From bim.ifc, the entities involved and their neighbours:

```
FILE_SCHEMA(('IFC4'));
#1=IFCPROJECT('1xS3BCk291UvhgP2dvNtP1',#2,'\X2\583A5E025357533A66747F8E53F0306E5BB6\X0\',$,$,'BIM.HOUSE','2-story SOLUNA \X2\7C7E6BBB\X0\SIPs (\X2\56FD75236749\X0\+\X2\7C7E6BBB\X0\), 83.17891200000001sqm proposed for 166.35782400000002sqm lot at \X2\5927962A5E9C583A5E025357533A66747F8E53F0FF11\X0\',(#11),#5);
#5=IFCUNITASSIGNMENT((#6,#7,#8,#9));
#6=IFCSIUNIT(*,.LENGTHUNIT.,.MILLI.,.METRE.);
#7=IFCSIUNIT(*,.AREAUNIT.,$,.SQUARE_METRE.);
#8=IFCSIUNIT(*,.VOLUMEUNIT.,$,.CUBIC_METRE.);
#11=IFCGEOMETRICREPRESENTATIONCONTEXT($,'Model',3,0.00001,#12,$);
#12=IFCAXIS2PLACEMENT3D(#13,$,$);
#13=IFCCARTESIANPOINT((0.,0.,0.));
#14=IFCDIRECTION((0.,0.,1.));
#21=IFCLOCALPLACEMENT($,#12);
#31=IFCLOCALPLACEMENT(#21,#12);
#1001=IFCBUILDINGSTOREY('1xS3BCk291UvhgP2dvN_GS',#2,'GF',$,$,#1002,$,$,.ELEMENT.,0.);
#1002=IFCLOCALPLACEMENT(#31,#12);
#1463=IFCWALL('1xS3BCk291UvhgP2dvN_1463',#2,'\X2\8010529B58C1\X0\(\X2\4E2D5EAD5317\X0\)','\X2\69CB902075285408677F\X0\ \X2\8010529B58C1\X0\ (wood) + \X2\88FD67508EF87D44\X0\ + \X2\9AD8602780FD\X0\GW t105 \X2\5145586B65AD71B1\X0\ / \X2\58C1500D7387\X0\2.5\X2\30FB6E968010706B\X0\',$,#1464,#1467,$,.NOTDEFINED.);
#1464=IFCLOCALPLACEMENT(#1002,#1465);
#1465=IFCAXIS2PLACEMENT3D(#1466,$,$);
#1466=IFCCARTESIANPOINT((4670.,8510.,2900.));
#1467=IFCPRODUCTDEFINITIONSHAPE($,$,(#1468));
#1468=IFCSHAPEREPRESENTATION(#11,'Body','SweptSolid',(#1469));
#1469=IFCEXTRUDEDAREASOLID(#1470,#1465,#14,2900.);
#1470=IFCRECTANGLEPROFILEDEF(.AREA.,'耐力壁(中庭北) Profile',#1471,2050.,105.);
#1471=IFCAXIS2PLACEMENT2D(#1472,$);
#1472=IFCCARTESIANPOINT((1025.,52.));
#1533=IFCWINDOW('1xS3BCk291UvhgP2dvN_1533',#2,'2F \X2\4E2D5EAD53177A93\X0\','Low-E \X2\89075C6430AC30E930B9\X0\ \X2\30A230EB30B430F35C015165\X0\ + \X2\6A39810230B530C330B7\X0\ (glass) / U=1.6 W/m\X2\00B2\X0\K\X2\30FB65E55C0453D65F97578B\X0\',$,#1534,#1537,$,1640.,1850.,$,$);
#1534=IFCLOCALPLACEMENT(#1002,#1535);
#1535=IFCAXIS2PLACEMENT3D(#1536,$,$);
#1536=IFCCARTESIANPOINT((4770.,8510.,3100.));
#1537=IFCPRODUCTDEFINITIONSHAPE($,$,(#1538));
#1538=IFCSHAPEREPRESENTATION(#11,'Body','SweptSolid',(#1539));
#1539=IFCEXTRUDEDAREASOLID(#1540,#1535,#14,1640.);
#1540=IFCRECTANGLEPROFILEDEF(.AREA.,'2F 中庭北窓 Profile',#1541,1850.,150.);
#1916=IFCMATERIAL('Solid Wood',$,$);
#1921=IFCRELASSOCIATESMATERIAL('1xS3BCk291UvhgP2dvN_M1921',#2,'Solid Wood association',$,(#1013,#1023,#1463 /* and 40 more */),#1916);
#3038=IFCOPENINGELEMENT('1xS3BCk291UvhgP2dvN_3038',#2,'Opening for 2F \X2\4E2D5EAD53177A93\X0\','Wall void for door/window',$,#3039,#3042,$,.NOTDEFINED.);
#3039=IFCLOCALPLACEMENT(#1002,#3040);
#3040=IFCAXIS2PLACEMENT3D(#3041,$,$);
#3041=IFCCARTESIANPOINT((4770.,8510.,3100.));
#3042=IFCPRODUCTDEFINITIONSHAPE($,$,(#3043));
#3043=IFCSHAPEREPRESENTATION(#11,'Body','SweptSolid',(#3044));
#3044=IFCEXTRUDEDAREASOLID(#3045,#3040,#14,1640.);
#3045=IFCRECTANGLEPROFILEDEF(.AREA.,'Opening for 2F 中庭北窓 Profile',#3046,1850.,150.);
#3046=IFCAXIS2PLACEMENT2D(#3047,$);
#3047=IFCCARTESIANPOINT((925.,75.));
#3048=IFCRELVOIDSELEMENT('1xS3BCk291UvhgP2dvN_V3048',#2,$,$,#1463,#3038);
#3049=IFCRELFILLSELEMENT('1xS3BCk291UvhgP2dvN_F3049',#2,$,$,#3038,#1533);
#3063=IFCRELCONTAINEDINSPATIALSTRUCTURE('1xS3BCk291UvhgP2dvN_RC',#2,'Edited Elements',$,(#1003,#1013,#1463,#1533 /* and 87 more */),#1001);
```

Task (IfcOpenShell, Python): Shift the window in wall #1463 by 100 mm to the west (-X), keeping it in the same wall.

```python
import ifcopenshell
import ifcopenshell.api.geometry
import ifcopenshell.util.placement

model = ifcopenshell.open("bim.ifc")

window = model.by_guid("1xS3BCk291UvhgP2dvN_1533")
opening = window.FillsVoids[0].RelatingOpeningElement
wall = opening.VoidsElements[0].RelatingBuildingElement

wall_matrix = ifcopenshell.util.placement.get_local_placement(wall.ObjectPlacement)
shift = wall_matrix[:3, 0] * -100.0
before = ifcopenshell.util.placement.get_local_placement(window.ObjectPlacement)[:3, 3].copy()

# The window is not placed relative to its opening, so move both.
for product in (opening, window):
    matrix = ifcopenshell.util.placement.get_local_placement(product.ObjectPlacement)
    matrix[:3, 3] += shift
    ifcopenshell.api.geometry.edit_object_placement(model, product=product, matrix=matrix, is_si=False)

after = ifcopenshell.util.placement.get_local_placement(window.ObjectPlacement)[:3, 3]
print("window moved by", (after - before).round(3) + 0.0)

model.write("bim_v2.ifc")
```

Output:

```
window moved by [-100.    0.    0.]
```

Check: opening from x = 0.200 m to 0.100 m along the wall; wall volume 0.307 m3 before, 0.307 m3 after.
